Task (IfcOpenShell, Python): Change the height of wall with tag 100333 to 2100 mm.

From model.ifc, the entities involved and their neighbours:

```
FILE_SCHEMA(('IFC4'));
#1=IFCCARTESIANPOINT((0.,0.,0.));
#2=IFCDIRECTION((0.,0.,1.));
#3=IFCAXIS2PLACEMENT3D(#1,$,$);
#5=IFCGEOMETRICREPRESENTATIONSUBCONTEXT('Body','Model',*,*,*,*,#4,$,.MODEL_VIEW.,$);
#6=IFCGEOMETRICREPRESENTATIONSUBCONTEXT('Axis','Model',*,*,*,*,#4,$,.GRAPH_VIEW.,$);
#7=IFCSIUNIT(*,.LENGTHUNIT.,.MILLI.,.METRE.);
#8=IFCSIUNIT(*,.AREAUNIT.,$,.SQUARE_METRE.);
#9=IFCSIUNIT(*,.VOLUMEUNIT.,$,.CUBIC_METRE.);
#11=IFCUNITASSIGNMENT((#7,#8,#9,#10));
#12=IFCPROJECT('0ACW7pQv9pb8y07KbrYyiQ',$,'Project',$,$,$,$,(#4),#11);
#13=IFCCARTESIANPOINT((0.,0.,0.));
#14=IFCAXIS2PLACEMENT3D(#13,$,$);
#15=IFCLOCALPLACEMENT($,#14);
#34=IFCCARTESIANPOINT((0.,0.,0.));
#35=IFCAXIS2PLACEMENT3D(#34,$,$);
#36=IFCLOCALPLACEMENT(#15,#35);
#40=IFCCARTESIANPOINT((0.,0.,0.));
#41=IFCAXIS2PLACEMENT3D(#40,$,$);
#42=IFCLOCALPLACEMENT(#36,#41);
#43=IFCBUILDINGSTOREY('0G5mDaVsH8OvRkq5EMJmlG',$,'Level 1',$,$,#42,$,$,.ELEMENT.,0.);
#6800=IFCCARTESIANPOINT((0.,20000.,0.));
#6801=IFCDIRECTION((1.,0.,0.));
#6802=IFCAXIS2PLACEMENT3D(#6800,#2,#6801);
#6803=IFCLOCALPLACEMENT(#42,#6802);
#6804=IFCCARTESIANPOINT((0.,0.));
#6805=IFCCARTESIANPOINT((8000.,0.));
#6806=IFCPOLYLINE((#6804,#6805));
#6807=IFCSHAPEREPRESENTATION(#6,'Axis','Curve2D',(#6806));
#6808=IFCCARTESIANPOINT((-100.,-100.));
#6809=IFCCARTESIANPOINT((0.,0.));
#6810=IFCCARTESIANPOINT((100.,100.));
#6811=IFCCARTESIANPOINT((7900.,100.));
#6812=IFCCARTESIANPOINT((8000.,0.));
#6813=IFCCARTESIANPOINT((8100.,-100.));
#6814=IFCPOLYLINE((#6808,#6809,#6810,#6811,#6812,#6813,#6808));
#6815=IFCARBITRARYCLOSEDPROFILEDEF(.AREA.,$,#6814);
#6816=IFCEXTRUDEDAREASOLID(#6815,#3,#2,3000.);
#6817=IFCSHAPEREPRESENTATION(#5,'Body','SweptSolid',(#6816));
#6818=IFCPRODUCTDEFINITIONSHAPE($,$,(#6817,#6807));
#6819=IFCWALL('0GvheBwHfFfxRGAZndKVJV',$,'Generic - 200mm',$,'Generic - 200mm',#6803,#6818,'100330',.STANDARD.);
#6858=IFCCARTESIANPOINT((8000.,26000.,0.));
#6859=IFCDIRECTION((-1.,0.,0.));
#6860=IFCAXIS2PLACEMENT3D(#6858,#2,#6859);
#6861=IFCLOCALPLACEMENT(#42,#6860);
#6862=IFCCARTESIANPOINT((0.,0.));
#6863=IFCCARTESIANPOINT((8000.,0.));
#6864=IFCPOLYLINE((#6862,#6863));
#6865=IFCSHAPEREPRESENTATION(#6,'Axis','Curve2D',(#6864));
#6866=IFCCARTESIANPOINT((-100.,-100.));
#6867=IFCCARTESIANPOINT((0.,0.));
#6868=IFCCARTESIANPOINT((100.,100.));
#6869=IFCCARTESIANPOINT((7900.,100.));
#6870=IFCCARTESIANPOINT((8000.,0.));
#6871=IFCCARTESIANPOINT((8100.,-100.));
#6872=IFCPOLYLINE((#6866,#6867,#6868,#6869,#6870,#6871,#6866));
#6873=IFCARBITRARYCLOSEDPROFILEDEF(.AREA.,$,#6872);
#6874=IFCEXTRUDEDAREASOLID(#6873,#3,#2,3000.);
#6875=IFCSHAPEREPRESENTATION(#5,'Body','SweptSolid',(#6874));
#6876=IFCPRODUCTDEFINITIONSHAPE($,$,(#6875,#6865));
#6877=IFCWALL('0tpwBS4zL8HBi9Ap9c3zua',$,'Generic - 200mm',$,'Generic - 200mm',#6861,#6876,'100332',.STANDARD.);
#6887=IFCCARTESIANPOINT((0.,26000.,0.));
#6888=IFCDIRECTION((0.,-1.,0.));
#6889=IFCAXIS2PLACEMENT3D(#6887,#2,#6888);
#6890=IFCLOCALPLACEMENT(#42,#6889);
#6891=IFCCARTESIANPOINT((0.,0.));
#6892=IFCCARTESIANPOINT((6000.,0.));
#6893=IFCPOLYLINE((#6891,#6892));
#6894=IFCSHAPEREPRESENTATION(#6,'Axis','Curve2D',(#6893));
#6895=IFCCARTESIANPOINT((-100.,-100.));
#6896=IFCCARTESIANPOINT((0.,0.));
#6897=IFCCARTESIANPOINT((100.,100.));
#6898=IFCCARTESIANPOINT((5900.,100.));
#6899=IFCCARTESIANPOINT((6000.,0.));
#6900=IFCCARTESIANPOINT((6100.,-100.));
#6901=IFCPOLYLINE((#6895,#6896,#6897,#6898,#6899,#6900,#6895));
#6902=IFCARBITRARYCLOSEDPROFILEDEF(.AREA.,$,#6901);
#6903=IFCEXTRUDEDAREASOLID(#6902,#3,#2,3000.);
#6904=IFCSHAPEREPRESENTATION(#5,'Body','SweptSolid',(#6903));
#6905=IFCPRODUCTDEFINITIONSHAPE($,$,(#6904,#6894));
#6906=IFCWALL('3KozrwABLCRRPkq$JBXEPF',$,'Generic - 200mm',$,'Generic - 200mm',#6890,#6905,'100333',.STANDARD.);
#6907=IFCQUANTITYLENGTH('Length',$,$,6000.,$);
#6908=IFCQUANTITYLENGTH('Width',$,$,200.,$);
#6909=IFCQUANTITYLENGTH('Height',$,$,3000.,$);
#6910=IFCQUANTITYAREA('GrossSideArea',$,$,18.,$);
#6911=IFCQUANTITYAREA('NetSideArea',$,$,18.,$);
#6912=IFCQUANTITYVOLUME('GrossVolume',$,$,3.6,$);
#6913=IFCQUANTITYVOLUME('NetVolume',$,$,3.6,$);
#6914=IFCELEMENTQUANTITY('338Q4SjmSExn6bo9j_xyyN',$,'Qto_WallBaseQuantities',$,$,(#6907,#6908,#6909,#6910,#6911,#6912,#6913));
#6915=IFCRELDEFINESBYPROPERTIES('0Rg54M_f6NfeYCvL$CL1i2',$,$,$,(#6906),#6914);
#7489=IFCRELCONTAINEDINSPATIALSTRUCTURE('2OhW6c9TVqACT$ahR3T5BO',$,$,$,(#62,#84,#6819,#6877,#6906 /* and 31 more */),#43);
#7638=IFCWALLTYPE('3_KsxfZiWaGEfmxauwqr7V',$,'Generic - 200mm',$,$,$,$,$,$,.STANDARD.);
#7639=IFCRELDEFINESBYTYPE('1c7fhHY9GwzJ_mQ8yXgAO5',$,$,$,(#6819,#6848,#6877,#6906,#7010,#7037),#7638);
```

```python
import ifcopenshell
import ifcopenshell.api.pset
import ifcopenshell.geom
import ifcopenshell.util.element
import ifcopenshell.util.representation
import ifcopenshell.util.shape
import ifcopenshell.util.unit

model = ifcopenshell.open("model.ifc")
unit_scale = ifcopenshell.util.unit.calculate_unit_scale(model)
area_scale = ifcopenshell.util.unit.calculate_unit_scale(model, "AREAUNIT")
volume_scale = ifcopenshell.util.unit.calculate_unit_scale(model, "VOLUMEUNIT")
settings = ifcopenshell.geom.settings()


def volume(element):
    """Net volume in cubic metres, openings subtracted."""
    shape = ifcopenshell.geom.create_shape(settings, element)
    return ifcopenshell.util.shape.get_volume(shape.geometry)


wall = model.by_id(6906)
before = volume(wall)

body = ifcopenshell.util.representation.get_representation(wall, "Model", "Body")
solid = body.Items[0]
old_height = solid.Depth
solid.Depth = 2.1 / unit_scale
after = volume(wall)
thickness = 0.2  # wall thickness in metres

# Update the stored height, areas and volumes.
qto = model.by_id(ifcopenshell.util.element.get_pset(wall, "Qto_WallBaseQuantities", should_inherit=False)["id"])
ifcopenshell.api.pset.edit_qto(model, qto=qto, properties={
    "Height": solid.Depth,
    "GrossSideArea": ifcopenshell.util.element.get_pset(wall, "Qto_WallBaseQuantities", "GrossSideArea") * solid.Depth / old_height,
    "NetSideArea": after / thickness / area_scale,
    "GrossVolume": ifcopenshell.util.element.get_pset(wall, "Qto_WallBaseQuantities", "GrossVolume") * solid.Depth / old_height,
    "NetVolume": after / volume_scale,
})

print(f"height {old_height:g} -> {solid.Depth:g}, volume {before:.3f} -> {after:.3f} m3")

model.write("model-out.ifc")
```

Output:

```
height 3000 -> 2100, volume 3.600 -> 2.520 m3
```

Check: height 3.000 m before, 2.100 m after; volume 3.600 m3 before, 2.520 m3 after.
